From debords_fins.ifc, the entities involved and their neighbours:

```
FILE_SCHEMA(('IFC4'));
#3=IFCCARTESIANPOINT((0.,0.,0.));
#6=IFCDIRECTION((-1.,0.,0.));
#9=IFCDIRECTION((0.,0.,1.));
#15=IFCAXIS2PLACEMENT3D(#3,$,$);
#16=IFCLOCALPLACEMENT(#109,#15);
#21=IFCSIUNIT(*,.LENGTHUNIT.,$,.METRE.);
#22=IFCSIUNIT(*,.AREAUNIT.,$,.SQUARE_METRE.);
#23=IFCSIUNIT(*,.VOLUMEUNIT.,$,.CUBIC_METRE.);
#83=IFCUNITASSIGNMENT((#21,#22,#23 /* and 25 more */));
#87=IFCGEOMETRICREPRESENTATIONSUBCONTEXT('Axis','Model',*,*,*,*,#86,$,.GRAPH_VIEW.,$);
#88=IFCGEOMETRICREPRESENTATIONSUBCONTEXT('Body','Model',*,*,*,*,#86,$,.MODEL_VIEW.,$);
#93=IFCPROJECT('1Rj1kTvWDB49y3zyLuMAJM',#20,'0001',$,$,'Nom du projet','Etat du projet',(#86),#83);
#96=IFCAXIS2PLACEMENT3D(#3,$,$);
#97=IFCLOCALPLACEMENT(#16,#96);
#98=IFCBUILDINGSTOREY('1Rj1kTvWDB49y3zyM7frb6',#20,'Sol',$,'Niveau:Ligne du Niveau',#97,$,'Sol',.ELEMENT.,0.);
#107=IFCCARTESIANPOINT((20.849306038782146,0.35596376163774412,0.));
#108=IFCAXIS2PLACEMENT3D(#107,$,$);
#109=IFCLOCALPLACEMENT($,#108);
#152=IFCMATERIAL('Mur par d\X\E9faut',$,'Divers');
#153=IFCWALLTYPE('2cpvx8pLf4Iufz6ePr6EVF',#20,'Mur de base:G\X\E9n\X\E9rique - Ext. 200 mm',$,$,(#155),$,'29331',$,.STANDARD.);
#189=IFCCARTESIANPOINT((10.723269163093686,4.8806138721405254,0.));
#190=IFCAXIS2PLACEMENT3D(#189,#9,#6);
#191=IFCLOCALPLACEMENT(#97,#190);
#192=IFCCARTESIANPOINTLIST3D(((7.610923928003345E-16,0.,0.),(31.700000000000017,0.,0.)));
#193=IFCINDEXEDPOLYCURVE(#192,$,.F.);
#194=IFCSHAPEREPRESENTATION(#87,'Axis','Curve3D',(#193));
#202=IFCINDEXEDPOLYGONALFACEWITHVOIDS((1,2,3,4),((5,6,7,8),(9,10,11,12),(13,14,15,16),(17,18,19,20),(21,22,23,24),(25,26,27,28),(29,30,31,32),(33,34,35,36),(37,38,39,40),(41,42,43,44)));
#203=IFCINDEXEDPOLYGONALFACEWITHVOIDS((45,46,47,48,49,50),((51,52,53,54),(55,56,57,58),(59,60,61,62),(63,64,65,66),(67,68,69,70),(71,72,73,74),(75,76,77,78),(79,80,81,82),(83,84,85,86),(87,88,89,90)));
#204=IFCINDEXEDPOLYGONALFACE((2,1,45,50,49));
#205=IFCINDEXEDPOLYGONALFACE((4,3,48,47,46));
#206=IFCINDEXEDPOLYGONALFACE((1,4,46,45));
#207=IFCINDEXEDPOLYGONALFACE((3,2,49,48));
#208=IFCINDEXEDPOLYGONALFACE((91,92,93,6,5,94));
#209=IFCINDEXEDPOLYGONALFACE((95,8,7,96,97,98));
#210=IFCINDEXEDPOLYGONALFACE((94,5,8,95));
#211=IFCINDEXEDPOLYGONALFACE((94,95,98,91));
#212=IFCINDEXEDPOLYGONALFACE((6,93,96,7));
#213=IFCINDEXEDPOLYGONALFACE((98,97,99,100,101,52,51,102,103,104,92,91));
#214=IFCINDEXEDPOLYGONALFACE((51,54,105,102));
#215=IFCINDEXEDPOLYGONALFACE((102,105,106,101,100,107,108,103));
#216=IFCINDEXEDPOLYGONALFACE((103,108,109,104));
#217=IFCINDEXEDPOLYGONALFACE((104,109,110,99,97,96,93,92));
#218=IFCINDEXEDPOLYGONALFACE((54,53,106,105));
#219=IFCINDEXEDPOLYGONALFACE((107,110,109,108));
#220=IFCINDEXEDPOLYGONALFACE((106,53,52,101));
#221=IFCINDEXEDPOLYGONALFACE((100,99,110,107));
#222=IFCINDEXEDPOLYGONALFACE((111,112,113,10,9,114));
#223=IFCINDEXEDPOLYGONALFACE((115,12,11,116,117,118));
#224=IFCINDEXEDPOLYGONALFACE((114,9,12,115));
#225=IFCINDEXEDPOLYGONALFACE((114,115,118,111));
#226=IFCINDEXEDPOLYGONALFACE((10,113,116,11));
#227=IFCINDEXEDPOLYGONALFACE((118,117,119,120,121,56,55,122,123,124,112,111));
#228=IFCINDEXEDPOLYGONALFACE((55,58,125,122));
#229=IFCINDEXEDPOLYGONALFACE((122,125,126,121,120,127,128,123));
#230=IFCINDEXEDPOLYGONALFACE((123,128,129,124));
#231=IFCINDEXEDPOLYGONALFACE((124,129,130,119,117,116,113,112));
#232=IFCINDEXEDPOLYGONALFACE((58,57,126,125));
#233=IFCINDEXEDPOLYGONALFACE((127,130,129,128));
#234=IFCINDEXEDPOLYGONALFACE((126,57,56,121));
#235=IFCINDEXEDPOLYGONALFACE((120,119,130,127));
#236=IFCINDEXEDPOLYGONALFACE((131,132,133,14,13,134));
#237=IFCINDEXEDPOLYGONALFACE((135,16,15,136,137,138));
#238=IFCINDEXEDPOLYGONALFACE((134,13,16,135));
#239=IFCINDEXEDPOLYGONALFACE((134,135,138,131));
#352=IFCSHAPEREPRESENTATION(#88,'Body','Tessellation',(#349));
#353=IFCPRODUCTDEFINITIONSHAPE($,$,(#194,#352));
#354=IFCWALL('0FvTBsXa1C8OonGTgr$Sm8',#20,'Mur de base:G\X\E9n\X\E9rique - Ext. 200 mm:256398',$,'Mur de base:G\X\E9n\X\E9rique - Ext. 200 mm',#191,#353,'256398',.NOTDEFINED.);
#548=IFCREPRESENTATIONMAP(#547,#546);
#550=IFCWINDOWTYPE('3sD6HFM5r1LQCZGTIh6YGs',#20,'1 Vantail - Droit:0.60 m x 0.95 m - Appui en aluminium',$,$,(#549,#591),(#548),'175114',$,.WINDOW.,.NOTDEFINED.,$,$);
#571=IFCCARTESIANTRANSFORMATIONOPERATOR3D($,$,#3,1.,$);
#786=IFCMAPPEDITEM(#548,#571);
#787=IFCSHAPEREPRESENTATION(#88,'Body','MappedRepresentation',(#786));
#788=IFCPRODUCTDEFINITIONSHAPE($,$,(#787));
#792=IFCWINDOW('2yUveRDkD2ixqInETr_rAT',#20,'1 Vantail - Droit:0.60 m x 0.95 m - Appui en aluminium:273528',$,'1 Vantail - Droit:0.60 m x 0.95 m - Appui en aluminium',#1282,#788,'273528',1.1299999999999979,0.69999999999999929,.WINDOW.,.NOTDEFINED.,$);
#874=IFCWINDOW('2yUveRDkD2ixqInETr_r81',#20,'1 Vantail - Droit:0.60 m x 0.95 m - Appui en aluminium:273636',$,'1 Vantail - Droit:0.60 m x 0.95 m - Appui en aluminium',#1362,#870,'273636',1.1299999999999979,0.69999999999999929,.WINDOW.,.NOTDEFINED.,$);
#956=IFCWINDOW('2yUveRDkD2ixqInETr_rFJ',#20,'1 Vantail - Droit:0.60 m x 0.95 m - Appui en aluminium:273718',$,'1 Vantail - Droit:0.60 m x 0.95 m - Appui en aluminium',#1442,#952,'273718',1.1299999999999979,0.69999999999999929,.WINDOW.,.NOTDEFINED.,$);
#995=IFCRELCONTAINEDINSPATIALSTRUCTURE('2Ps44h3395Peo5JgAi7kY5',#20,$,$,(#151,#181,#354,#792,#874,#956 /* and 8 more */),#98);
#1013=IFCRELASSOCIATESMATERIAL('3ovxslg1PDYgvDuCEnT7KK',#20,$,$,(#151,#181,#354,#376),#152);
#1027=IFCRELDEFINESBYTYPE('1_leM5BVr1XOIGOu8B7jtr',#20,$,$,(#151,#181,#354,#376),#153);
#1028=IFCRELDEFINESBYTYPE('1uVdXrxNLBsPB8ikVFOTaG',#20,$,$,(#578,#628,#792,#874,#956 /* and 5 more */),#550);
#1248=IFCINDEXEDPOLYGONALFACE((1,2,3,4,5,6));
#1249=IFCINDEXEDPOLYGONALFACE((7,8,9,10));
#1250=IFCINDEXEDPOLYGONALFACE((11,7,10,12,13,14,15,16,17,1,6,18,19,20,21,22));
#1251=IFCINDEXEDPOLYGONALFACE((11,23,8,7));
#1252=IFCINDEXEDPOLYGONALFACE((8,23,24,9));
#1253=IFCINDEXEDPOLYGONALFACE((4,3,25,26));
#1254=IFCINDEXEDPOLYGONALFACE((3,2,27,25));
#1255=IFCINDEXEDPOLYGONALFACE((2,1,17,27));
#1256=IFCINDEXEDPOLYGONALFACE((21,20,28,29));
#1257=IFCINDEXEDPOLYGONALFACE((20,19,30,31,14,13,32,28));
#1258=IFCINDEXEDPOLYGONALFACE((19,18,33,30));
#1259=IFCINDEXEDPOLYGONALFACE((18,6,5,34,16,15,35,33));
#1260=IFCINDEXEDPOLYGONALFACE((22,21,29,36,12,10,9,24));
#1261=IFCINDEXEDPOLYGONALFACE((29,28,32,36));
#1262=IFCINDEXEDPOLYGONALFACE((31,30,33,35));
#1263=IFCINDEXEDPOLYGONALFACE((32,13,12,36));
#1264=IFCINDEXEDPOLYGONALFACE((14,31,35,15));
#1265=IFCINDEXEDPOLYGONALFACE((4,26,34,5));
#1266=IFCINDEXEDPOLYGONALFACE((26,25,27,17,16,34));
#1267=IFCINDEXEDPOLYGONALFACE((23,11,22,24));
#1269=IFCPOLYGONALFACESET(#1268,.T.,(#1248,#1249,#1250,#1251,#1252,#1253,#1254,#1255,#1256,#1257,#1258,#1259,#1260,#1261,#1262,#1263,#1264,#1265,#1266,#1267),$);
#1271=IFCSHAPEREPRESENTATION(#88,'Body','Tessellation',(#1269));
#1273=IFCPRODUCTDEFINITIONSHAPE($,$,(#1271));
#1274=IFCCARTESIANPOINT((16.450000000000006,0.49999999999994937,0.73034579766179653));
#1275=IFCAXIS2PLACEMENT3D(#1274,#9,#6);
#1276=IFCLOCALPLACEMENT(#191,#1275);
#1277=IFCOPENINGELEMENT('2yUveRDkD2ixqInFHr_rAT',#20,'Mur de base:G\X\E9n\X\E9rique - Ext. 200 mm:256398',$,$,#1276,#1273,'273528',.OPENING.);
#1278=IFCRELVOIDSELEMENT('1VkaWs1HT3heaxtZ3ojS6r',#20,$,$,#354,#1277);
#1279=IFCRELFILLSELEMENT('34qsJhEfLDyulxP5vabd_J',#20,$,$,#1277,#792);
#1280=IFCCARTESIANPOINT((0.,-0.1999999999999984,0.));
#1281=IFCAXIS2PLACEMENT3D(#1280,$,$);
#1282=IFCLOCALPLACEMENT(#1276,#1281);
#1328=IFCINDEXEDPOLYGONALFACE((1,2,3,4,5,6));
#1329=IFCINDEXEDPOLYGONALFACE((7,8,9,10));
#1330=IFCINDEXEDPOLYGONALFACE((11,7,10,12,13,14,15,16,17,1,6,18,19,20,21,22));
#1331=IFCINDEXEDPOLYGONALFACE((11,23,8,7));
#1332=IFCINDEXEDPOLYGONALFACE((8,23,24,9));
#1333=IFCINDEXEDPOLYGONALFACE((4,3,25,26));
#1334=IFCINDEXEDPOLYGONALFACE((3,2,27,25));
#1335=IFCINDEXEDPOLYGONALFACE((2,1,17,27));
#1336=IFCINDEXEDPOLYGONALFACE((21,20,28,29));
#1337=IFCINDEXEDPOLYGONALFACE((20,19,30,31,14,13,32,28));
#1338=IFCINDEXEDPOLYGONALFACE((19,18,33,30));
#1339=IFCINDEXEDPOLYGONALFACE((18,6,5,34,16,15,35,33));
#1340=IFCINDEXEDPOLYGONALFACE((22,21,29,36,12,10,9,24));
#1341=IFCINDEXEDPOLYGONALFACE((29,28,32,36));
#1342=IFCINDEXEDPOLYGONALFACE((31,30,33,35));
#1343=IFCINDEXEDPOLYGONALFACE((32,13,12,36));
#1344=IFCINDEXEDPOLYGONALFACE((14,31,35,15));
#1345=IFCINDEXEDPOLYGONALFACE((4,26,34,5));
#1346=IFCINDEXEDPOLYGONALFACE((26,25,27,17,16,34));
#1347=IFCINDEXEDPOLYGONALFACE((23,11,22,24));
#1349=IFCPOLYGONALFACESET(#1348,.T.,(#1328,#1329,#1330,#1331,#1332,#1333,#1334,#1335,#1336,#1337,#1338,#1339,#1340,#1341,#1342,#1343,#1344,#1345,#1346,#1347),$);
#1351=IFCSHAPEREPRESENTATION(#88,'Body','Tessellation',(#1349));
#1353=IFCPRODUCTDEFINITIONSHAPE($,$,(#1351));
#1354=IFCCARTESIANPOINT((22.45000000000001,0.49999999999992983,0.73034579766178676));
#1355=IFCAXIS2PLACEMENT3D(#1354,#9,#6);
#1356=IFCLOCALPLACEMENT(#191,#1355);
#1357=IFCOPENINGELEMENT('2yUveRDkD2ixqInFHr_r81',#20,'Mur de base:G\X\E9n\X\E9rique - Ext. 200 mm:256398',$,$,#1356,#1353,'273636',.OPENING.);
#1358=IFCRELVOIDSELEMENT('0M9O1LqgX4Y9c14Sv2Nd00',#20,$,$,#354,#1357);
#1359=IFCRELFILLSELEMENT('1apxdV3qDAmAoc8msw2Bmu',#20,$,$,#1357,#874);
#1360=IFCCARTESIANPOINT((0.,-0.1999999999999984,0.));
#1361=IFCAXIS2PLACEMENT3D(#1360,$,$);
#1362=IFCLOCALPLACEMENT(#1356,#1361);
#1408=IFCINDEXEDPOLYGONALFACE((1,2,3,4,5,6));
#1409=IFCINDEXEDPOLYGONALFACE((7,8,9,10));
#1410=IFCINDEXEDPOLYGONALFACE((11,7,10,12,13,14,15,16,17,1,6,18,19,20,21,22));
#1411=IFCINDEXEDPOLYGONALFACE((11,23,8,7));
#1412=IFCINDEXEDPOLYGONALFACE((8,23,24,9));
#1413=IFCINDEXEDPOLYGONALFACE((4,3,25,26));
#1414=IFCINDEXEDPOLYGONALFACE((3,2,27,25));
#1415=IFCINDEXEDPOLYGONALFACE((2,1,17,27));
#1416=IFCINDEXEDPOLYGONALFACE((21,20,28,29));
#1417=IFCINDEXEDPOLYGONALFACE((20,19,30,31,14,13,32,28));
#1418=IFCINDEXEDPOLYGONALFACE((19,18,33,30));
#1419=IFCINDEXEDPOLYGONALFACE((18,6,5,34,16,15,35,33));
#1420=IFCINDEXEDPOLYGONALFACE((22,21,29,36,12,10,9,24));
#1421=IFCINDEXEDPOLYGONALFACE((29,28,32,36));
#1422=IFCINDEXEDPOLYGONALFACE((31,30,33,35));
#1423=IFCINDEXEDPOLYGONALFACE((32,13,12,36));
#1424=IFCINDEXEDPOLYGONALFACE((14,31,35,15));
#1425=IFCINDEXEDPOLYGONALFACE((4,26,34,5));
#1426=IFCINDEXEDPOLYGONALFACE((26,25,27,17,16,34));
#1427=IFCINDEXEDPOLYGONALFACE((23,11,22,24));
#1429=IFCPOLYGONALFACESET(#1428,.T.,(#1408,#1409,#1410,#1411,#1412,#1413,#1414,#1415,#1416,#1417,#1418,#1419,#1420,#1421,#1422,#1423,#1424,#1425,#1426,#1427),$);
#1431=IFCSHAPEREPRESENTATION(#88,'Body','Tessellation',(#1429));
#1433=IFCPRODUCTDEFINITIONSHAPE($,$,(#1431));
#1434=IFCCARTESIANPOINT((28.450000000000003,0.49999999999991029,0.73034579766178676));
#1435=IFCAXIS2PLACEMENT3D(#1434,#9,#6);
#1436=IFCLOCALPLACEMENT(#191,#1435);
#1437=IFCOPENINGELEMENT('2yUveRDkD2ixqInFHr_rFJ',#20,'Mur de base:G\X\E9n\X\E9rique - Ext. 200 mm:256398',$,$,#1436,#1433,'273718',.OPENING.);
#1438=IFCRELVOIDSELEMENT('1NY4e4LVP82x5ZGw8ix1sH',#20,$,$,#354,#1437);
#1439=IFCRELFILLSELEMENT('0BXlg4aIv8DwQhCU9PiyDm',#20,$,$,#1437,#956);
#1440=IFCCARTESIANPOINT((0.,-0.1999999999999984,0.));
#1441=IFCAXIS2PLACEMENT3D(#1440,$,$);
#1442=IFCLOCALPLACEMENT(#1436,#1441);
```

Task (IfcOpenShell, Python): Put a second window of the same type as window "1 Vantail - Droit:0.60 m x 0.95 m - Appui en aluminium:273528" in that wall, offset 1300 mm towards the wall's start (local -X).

```python
import ifcopenshell
import ifcopenshell.api.feature
import ifcopenshell.api.geometry
import ifcopenshell.api.root
import ifcopenshell.geom
import ifcopenshell.util.element
import ifcopenshell.util.placement
import ifcopenshell.util.shape
import ifcopenshell.util.unit

model = ifcopenshell.open("debords_fins.ifc")
unit_scale = ifcopenshell.util.unit.calculate_unit_scale(model)
settings = ifcopenshell.geom.settings()


def volume(element):
    """Net volume in cubic metres, openings subtracted."""
    shape = ifcopenshell.geom.create_shape(settings, element)
    return ifcopenshell.util.shape.get_volume(shape.geometry)


def reuse_history(source, copy):
    """copy_class also copies each property set's owner history, people and application; keep the originals."""
    for rel in copy.IsDefinedBy:
        if rel.is_a("IfcRelDefinesByProperties") and (history := rel.RelatingPropertyDefinition.OwnerHistory):
            rel.RelatingPropertyDefinition.OwnerHistory = source.OwnerHistory
            ifcopenshell.util.element.remove_deep2(model, history)


window = model.by_guid("2yUveRDkD2ixqInETr_rAT")
opening = window.FillsVoids[0].RelatingOpeningElement
wall = opening.VoidsElements[0].RelatingBuildingElement
before = volume(wall)
shift = ifcopenshell.util.placement.get_local_placement(wall.ObjectPlacement)[:3, 0] * -1.3 / unit_scale

# copy_class copies the void relationship, type, container and properties, but no geometry.
new_opening = ifcopenshell.api.root.copy_class(model, product=opening)
new_opening.Representation = ifcopenshell.util.element.copy_deep(
    model, opening.Representation, exclude=["IfcGeometricRepresentationContext", "IfcRepresentationMap"]
)
new_opening.Name = "Mur de base:Générique - Ext. 200 mm"
new_opening.Tag = None
new_window = ifcopenshell.api.root.copy_class(model, product=window)
new_window.Representation = ifcopenshell.util.element.copy_deep(
    model, window.Representation, exclude=["IfcGeometricRepresentationContext", "IfcRepresentationMap"]
)
new_window.Name = "1 Vantail - Droit:0.60 m x 0.95 m - Appui en aluminium"
new_window.Tag = None
reuse_history(window, new_window)
ifcopenshell.api.feature.add_filling(model, opening=new_opening, element=new_window)

for old, new in ((opening, new_opening), (window, new_window)):
    matrix = ifcopenshell.util.placement.get_local_placement(old.ObjectPlacement)
    matrix[:3, 3] += shift
    ifcopenshell.api.geometry.edit_object_placement(model, product=new, matrix=matrix, is_si=False)

after = volume(wall)

print(f"wall volume {before:.3f} -> {after:.3f} m3")

model.write("debords_fins_v2.ifc")
```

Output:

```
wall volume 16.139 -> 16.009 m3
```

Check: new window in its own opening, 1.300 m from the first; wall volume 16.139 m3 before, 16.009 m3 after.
